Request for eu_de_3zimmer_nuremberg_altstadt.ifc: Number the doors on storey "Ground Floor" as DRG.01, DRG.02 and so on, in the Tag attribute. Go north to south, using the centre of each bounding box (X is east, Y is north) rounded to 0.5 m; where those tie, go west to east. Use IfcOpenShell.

First a look at what the model holds.

```python
import ifcopenshell
import ifcopenshell.util.element
import ifcopenshell.util.placement

model = ifcopenshell.open("eu_de_3zimmer_nuremberg_altstadt.ifc")
print(model.schema)
storey = next(s for s in model.by_type("IfcBuildingStorey") if s.Name == "Ground Floor")
doors = [e for e in ifcopenshell.util.element.get_decomposition(storey) if e.is_a("IfcDoor")]
for e in sorted(doors, key=lambda e: e.id()):
    origin = ifcopenshell.util.placement.get_local_placement(e.ObjectPlacement)[:3, 3]
    print(e.id(), e.Tag, e.Name, origin.round(2) + 0.0, sep=" | ")
```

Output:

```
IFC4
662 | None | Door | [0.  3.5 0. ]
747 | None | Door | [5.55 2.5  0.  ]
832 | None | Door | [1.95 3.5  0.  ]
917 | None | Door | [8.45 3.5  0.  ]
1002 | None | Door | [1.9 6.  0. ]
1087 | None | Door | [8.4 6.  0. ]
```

```python
import ifcopenshell
import ifcopenshell.geom
import ifcopenshell.util.element
import ifcopenshell.util.shape

model = ifcopenshell.open("eu_de_3zimmer_nuremberg_altstadt.ifc")
settings = ifcopenshell.geom.settings()
settings.set("use-world-coords", True)


def centre(element):
    shape = ifcopenshell.geom.create_shape(settings, element)
    return ifcopenshell.util.shape.get_bbox_centroid(shape.geometry)


storey = next(s for s in model.by_type("IfcBuildingStorey") if s.Name == "Ground Floor")
doors = [e for e in ifcopenshell.util.element.get_decomposition(storey) if e.is_a("IfcDoor")]

# Insertion points can sit at a corner or the storey origin, so sort by the geometry (in metres).
centres = {e: centre(e) for e in doors}
doors.sort(key=lambda e: (-round(centres[e][1] / 0.5), centres[e][0]))

for i, e in enumerate(doors, start=1):
    number = f"DRG.{i:02d}"
    e.Tag = number
    print(e.id(), number)

model.write("eu_de_3zimmer_nuremberg_altstadt_rev.ifc")
```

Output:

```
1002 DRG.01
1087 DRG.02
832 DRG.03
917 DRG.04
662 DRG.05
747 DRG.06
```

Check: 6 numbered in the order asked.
